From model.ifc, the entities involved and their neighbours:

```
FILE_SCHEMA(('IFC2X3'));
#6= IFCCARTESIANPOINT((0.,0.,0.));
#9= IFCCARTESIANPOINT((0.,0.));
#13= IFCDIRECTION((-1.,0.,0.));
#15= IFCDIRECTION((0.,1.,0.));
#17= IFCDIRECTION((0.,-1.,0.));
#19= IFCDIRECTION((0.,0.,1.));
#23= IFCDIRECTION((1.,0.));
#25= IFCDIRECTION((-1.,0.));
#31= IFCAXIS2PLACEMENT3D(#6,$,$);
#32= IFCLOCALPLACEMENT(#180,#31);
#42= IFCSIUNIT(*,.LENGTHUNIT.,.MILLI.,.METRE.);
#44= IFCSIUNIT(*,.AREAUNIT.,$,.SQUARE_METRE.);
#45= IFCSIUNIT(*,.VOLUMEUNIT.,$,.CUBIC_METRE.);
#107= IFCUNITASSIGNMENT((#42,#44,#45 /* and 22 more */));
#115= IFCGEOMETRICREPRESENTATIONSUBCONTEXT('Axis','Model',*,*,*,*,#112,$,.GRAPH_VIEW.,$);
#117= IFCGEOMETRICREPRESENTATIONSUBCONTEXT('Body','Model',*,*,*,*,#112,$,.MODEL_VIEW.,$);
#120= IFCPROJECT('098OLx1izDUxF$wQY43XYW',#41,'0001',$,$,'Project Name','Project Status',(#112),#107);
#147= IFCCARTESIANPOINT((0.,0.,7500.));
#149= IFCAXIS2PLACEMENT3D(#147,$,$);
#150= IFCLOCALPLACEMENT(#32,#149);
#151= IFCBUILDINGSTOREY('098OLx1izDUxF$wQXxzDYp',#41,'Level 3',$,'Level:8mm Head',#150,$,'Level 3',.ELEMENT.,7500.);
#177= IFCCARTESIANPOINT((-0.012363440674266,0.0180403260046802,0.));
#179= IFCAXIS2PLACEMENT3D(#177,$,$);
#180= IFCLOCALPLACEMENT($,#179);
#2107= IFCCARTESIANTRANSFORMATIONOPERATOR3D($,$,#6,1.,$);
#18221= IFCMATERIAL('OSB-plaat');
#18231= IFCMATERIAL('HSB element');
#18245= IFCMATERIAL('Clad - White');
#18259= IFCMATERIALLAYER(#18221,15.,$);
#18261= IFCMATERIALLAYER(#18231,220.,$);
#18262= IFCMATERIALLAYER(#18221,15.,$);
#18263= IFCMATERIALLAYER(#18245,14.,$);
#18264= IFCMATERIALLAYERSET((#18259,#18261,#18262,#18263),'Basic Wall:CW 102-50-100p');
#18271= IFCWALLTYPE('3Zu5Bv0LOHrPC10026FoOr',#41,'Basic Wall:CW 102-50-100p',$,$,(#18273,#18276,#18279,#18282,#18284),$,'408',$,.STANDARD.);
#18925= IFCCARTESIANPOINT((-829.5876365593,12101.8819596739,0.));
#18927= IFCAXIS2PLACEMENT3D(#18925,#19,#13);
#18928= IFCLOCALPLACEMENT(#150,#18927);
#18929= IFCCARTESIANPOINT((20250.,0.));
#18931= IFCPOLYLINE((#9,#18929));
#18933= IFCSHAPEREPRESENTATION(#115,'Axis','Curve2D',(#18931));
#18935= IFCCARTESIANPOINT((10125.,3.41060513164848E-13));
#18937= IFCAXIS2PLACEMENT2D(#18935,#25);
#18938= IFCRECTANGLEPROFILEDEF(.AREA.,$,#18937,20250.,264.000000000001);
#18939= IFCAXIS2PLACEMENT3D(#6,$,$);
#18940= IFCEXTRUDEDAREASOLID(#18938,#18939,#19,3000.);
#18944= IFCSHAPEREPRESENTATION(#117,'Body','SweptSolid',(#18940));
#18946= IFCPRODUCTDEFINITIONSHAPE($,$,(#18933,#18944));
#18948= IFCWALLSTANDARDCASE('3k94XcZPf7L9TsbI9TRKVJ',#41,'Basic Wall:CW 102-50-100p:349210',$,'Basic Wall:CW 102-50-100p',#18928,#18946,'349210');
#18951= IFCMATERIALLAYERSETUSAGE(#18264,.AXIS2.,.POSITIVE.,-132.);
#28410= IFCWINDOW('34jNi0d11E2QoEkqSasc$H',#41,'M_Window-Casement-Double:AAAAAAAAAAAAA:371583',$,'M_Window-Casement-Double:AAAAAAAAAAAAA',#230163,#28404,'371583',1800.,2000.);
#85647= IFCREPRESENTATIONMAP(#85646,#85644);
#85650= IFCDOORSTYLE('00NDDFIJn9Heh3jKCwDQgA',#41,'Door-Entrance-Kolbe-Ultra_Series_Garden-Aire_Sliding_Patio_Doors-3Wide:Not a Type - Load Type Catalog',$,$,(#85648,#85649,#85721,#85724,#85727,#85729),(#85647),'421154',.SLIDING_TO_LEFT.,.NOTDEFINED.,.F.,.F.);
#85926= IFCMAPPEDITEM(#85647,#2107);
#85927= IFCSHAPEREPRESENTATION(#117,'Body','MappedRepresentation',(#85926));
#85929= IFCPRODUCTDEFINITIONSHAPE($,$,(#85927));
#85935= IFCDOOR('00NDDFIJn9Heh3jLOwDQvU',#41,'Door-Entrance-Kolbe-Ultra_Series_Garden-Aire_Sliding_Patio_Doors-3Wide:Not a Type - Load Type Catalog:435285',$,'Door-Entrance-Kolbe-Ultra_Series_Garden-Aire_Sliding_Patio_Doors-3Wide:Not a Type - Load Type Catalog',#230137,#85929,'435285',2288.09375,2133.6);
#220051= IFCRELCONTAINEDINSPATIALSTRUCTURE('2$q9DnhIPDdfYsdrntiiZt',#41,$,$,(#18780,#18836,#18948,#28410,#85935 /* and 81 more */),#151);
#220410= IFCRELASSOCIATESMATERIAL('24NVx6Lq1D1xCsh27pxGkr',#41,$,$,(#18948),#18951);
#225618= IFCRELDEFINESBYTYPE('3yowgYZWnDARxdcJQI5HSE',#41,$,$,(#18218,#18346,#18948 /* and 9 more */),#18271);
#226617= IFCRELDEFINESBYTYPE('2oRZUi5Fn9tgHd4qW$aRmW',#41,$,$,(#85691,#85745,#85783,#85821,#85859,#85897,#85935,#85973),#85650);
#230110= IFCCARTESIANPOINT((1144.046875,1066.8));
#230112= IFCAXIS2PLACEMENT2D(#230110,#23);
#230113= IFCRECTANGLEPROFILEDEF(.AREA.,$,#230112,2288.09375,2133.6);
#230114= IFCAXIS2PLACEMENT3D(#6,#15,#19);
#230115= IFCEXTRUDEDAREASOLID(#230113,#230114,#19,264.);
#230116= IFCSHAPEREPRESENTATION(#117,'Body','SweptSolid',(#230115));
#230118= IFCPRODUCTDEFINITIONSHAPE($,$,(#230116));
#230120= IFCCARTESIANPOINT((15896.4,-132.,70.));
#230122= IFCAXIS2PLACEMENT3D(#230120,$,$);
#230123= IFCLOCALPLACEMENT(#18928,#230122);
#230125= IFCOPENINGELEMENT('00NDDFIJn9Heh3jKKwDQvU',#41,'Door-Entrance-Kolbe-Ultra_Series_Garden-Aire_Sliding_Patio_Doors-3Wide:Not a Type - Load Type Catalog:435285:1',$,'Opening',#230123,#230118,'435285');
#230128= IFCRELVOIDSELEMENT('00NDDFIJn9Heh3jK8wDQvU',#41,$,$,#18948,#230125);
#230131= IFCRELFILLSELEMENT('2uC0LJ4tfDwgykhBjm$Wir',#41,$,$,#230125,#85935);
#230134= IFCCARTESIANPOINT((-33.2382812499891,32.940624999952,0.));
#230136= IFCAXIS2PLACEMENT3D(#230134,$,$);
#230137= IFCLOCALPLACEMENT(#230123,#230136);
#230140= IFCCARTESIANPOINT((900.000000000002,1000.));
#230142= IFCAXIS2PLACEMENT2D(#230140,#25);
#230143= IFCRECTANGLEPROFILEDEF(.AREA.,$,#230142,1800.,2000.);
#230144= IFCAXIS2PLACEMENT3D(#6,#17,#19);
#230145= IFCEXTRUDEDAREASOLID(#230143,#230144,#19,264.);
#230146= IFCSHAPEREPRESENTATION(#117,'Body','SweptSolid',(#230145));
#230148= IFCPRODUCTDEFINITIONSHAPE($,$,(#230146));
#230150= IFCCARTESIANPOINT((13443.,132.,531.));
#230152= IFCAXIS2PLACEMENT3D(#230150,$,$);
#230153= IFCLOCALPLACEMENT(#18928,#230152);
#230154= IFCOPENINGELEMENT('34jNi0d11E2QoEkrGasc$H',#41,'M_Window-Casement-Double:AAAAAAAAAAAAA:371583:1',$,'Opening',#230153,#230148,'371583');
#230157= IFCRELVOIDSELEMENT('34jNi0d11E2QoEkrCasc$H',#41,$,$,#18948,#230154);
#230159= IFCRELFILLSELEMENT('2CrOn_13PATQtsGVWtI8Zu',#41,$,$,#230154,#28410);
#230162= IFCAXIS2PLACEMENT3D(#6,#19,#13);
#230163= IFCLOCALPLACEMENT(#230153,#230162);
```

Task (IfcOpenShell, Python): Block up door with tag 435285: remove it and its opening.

```python
import ifcopenshell
import ifcopenshell.api.feature
import ifcopenshell.api.root
import ifcopenshell.geom
import ifcopenshell.util.shape

model = ifcopenshell.open("model.ifc")
settings = ifcopenshell.geom.settings()


def volume(element):
    """Net volume in cubic metres, openings subtracted."""
    shape = ifcopenshell.geom.create_shape(settings, element)
    return ifcopenshell.util.shape.get_volume(shape.geometry)


door = model.by_guid("00NDDFIJn9Heh3jLOwDQvU")
opening = door.FillsVoids[0].RelatingOpeningElement
wall = opening.VoidsElements[0].RelatingBuildingElement
before = volume(wall)

ifcopenshell.api.root.remove_product(model, product=door)
ifcopenshell.api.feature.remove_feature(model, feature=opening)

after = volume(wall)

print(f"wall volume {before:.3f} -> {after:.3f} m3")

model.write("model-out.ifc")
```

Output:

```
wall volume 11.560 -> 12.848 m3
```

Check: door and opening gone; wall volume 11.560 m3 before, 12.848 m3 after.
